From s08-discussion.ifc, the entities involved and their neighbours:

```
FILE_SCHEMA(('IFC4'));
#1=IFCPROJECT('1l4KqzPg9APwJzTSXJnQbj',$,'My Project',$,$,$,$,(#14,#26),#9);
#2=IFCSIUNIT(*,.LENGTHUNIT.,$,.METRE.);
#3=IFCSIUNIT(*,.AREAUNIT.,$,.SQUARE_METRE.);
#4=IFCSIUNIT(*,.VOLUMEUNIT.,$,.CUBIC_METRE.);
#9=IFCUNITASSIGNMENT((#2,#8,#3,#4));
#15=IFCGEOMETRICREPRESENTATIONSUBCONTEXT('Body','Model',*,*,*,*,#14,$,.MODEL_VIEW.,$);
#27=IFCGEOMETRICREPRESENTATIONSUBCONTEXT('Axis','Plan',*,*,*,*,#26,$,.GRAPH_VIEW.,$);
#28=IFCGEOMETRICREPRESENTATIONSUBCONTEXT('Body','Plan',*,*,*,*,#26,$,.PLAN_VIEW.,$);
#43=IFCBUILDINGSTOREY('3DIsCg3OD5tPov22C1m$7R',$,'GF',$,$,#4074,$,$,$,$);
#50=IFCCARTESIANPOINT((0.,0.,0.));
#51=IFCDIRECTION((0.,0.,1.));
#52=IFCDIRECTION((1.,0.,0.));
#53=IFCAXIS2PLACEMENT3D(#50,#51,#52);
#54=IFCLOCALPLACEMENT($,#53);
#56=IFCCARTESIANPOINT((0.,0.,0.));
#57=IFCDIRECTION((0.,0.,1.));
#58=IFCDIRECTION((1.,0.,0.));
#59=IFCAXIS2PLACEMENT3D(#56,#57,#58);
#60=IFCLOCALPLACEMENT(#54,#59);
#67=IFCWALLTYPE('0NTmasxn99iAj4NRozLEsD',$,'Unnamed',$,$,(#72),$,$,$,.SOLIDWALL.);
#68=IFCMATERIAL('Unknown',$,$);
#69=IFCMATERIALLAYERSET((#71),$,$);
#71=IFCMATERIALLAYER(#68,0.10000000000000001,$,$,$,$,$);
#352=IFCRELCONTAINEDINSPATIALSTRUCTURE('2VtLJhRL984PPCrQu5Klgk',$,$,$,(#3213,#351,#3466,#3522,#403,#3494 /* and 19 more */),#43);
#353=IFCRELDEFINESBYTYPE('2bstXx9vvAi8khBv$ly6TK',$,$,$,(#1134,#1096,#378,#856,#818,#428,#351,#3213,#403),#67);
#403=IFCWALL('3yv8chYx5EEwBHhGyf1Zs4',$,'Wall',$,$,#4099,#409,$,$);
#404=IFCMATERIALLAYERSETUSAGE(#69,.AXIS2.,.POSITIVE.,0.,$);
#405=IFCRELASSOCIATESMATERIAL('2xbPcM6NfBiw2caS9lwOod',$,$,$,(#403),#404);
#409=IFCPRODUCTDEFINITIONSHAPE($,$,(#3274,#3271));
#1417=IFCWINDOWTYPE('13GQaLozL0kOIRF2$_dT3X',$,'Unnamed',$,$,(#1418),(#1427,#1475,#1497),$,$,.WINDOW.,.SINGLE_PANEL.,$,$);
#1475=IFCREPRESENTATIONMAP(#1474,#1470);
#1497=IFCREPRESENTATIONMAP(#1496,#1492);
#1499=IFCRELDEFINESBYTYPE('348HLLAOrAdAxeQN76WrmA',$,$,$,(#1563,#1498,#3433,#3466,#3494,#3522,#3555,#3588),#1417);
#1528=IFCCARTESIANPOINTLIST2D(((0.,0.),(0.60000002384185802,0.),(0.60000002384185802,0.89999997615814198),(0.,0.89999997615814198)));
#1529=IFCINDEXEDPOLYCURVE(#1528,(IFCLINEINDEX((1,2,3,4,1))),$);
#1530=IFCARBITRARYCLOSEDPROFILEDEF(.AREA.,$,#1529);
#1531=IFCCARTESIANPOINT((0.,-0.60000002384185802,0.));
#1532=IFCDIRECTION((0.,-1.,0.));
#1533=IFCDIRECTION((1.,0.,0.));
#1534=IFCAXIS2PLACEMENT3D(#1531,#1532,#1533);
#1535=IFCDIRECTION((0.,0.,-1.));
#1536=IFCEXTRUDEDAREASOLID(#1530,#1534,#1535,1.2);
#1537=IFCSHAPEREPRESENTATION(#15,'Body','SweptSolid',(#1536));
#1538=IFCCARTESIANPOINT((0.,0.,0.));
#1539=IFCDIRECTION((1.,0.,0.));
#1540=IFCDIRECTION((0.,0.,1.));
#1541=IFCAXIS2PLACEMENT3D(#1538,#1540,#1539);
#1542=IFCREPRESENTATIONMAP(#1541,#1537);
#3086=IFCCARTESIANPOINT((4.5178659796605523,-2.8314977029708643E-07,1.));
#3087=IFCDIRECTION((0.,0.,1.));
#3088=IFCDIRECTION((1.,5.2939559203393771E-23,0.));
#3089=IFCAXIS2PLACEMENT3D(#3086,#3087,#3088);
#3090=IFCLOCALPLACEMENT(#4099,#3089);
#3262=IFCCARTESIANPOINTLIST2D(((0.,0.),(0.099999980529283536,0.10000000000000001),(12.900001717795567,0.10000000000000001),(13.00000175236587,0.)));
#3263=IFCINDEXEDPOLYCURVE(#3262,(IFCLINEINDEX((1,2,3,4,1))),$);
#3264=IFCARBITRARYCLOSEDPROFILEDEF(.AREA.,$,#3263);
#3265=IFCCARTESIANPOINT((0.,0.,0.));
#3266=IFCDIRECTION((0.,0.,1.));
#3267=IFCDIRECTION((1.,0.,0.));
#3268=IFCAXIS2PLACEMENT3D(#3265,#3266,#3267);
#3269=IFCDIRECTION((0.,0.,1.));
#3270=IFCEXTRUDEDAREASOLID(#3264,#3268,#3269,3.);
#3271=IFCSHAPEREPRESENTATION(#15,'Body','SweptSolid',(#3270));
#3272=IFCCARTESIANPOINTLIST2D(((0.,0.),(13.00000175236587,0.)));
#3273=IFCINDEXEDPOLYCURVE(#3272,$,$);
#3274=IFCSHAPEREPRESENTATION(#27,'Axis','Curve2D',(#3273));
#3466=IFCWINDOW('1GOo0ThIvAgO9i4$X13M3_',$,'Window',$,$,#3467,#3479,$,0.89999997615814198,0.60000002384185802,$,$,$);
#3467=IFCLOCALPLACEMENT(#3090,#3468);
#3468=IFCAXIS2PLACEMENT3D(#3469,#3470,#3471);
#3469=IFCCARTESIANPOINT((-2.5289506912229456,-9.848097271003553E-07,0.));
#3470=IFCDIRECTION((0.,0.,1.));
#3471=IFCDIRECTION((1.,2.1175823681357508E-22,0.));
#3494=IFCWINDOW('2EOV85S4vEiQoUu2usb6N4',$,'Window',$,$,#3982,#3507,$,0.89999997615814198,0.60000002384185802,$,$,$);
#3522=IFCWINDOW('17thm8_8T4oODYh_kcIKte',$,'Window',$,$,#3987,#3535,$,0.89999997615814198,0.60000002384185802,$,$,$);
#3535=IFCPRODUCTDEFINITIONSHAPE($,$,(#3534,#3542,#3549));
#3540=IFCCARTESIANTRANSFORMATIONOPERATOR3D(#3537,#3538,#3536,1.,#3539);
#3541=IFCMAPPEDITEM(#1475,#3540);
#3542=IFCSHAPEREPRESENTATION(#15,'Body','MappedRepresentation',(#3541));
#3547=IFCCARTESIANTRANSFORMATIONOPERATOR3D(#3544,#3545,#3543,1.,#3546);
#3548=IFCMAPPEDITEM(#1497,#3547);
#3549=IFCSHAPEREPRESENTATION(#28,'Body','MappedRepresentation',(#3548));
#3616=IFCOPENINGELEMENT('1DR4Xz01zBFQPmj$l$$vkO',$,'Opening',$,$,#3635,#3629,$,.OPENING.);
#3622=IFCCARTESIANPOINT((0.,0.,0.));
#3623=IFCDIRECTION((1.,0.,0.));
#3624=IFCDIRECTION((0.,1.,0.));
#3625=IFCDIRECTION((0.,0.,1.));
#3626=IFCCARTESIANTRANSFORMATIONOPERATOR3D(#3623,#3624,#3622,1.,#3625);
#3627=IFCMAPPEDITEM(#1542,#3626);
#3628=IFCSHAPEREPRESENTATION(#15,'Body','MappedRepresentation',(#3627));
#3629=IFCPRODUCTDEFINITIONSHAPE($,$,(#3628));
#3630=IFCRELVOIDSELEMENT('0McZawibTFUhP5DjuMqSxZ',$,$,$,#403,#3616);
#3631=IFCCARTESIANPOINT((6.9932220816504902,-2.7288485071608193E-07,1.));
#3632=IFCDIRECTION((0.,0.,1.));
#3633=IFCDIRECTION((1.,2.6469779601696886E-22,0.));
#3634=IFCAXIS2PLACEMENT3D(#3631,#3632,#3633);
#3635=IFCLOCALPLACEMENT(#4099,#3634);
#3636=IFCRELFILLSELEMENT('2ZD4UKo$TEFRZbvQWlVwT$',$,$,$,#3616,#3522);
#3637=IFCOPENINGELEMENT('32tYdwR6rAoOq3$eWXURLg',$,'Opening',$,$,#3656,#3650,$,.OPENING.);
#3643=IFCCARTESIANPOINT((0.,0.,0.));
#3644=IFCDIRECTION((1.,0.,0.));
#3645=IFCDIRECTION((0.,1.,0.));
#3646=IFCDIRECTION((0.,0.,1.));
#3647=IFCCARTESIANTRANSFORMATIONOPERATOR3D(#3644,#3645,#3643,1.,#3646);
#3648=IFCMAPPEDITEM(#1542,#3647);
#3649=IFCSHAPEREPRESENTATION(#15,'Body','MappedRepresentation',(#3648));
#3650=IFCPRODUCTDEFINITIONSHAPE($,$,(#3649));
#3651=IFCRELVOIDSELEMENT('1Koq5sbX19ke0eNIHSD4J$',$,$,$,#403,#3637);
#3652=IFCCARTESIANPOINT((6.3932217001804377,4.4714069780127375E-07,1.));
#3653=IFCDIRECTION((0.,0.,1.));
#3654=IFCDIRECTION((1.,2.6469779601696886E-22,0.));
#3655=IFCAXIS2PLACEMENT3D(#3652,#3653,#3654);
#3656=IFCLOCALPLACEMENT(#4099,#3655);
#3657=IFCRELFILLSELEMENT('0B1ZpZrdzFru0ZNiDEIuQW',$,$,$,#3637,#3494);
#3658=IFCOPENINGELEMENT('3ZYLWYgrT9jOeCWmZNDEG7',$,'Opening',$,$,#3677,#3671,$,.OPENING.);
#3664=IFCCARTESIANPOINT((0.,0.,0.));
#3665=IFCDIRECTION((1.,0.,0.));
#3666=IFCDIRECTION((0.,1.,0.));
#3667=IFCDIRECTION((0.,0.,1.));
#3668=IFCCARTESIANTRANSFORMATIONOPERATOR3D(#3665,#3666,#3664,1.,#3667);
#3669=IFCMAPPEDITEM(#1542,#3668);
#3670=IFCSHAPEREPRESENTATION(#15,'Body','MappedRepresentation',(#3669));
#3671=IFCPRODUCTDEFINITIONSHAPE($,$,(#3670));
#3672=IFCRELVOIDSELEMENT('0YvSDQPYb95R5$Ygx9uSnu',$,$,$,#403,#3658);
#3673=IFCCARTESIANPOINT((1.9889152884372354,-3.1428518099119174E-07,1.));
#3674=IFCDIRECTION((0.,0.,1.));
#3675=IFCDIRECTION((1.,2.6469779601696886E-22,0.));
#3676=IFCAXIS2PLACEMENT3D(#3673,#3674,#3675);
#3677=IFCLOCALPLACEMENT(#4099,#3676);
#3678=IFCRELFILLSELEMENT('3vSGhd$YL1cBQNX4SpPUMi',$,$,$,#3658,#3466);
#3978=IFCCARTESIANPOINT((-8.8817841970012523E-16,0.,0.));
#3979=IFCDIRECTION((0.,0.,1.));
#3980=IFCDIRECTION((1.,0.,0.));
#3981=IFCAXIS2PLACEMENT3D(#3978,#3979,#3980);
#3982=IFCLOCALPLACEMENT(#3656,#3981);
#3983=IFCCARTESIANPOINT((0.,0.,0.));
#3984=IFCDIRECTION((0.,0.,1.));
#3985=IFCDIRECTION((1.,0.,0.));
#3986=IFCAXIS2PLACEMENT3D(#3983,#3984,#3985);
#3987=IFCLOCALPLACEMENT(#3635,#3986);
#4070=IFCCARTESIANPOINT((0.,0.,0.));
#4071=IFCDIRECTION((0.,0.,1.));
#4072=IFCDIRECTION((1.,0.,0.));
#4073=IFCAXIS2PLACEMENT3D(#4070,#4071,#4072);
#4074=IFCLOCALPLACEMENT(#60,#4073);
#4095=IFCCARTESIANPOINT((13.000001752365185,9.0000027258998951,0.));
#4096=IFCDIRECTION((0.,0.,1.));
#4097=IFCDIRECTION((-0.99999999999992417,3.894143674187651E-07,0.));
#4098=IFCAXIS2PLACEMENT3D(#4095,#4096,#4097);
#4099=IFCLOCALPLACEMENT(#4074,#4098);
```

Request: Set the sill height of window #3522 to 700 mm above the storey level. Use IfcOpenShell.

```python
import numpy as np
import ifcopenshell
import ifcopenshell.api.geometry
import ifcopenshell.geom
import ifcopenshell.util.element
import ifcopenshell.util.placement
import ifcopenshell.util.shape
import ifcopenshell.util.unit

model = ifcopenshell.open("s08-discussion.ifc")
unit_scale = ifcopenshell.util.unit.calculate_unit_scale(model)

window = model.by_id(3522)
opening = window.FillsVoids[0].RelatingOpeningElement
storey = ifcopenshell.util.element.get_container(window, ifc_class="IfcBuildingStorey")
level = ifcopenshell.util.placement.get_local_placement(storey.ObjectPlacement)[2, 3]

# The opening's origin need not be at the sill, so measure its lowest point.
shape = ifcopenshell.geom.create_shape(ifcopenshell.geom.settings(), opening)
bottom = ifcopenshell.util.shape.get_shape_bottom_elevation(shape, shape.geometry) / unit_scale
dz = level + 0.7 - bottom

shift = np.array([0.0, 0.0, dz])
# The window is placed relative to its opening, so it follows when the opening moves.
matrix = ifcopenshell.util.placement.get_local_placement(opening.ObjectPlacement)
matrix[:3, 3] += shift
ifcopenshell.api.geometry.edit_object_placement(
    model, product=opening, matrix=matrix, is_si=False, should_transform_children=True
)

print(f"moved by {dz * unit_scale:+.3f} m")

model.write("s08-discussion-out.ifc")
```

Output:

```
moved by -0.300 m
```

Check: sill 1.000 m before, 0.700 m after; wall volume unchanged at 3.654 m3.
